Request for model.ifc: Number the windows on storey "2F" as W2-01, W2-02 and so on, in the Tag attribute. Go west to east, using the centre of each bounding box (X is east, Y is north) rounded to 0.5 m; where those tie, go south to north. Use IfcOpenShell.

First a look at what the model holds.

```python
import ifcopenshell
import ifcopenshell.util.element
import ifcopenshell.util.placement

model = ifcopenshell.open("model.ifc")
print(model.schema)
storey = next(s for s in model.by_type("IfcBuildingStorey") if s.Name == "2F")
windows = [e for e in ifcopenshell.util.element.get_decomposition(storey) if e.is_a("IfcWindow")]
for e in sorted(windows, key=lambda e: e.id()):
    origin = ifcopenshell.util.placement.get_local_placement(e.ObjectPlacement)[:3, 3]
    print(e.id(), e.Tag, e.Name, origin.round(2) + 0.0, sep=" | ")
```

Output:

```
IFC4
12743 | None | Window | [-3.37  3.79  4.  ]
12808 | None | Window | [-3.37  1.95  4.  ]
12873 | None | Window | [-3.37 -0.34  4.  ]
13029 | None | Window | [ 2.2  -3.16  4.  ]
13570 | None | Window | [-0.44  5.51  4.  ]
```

```python
import ifcopenshell
import ifcopenshell.geom
import ifcopenshell.util.element
import ifcopenshell.util.shape

model = ifcopenshell.open("model.ifc")
settings = ifcopenshell.geom.settings()
settings.set("use-world-coords", True)


def centre(element):
    shape = ifcopenshell.geom.create_shape(settings, element)
    return ifcopenshell.util.shape.get_bbox_centroid(shape.geometry)


storey = next(s for s in model.by_type("IfcBuildingStorey") if s.Name == "2F")
windows = [e for e in ifcopenshell.util.element.get_decomposition(storey) if e.is_a("IfcWindow")]

# Insertion points can sit at a corner or the storey origin, so sort by the geometry (in metres).
centres = {e: centre(e) for e in windows}
windows.sort(key=lambda e: (round(centres[e][0] / 0.5), centres[e][1]))

for i, e in enumerate(windows, start=1):
    number = f"W2-{i:02d}"
    e.Tag = number
    print(e.id(), number)

model.write("model-out.ifc")
```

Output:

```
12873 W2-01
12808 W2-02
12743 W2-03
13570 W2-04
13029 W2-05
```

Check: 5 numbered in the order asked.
